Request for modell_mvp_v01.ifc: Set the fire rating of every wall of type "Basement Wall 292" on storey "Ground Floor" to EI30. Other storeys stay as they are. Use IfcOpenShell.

First a look at what the model holds.

```python
import ifcopenshell
import ifcopenshell.util.element

model = ifcopenshell.open("modell_mvp_v01.ifc")
print(model.schema)
storey = next(s for s in model.by_type("IfcBuildingStorey") if s.Name == "Ground Floor")
walls = [e for e in ifcopenshell.util.element.get_decomposition(storey) if e.is_a("IfcWall")]
seen = {}
for e in walls:
    element_type = ifcopenshell.util.element.get_type(e)
    key = (element_type.Name if element_type != e and element_type else None, ifcopenshell.util.element.get_pset(e, "Pset_WallCommon", "FireRating"))
    seen[key] = seen.get(key, 0) + 1
for (name, value), count in sorted(seen.items(), key=str):
    print(count, "x", name, "|", value)
```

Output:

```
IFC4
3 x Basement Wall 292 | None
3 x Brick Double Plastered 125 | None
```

```python
import ifcopenshell
import ifcopenshell.api.pset
import ifcopenshell.util.element

model = ifcopenshell.open("modell_mvp_v01.ifc")

storey = next(s for s in model.by_type("IfcBuildingStorey") if s.Name == "Ground Floor")
walls = [e for e in ifcopenshell.util.element.get_decomposition(storey) if e.is_a("IfcWall")]

count = 0
for e in walls:
    element_type = ifcopenshell.util.element.get_type(e)
    if element_type in (None, e) or element_type.Name != "Basement Wall 292":
        continue
    # add_pset returns the element's existing set when there is one.
    pset = ifcopenshell.api.pset.add_pset(model, product=e, name="Pset_WallCommon")
    ifcopenshell.api.pset.edit_pset(model, pset=pset, properties={"FireRating": "EI30"})
    count += 1

print(count, "walls updated")

model.write("modell_mvp_v01_v2.ifc")
```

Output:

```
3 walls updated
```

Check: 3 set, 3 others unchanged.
